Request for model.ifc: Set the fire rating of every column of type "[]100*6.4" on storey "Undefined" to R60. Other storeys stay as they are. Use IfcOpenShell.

First a look at what the model holds.

```python
import ifcopenshell
import ifcopenshell.util.element

model = ifcopenshell.open("model.ifc")
print(model.schema)
storey = next(s for s in model.by_type("IfcBuildingStorey") if s.Name == "Undefined")
columns = [e for e in ifcopenshell.util.element.get_decomposition(storey) if e.is_a("IfcColumn")]
seen = {}
for e in columns:
    element_type = ifcopenshell.util.element.get_type(e)
    key = (element_type.Name if element_type != e and element_type else None, ifcopenshell.util.element.get_pset(e, "Pset_ColumnCommon", "FireRating"))
    seen[key] = seen.get(key, 0) + 1
for (name, value), count in sorted(seen.items(), key=str):
    print(count, "x", name, "|", value)
```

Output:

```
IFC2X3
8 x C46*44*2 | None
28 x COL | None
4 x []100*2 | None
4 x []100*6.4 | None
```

```python
import ifcopenshell
import ifcopenshell.api.pset
import ifcopenshell.util.element

model = ifcopenshell.open("model.ifc")

storey = next(s for s in model.by_type("IfcBuildingStorey") if s.Name == "Undefined")
columns = [e for e in ifcopenshell.util.element.get_decomposition(storey) if e.is_a("IfcColumn")]

count = 0
for e in columns:
    element_type = ifcopenshell.util.element.get_type(e)
    if element_type in (None, e) or element_type.Name != "[]100*6.4":
        continue
    found = ifcopenshell.util.element.get_pset(e, "Pset_ColumnCommon", should_inherit=False)
    if found:
        pset = model.by_id(found["id"])
        if len(ifcopenshell.util.element.get_elements_by_pset(pset)) > 1:
            pset = ifcopenshell.api.pset.unshare_pset(model, products=[e], pset=pset)[0]
    else:
        pset = ifcopenshell.api.pset.add_pset(model, product=e, name="Pset_ColumnCommon")
    ifcopenshell.api.pset.edit_pset(model, pset=pset, properties={"FireRating": "R60"})
    count += 1

print(count, "columns updated")

model.write("model_updated.ifc")
```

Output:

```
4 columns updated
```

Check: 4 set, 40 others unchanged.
